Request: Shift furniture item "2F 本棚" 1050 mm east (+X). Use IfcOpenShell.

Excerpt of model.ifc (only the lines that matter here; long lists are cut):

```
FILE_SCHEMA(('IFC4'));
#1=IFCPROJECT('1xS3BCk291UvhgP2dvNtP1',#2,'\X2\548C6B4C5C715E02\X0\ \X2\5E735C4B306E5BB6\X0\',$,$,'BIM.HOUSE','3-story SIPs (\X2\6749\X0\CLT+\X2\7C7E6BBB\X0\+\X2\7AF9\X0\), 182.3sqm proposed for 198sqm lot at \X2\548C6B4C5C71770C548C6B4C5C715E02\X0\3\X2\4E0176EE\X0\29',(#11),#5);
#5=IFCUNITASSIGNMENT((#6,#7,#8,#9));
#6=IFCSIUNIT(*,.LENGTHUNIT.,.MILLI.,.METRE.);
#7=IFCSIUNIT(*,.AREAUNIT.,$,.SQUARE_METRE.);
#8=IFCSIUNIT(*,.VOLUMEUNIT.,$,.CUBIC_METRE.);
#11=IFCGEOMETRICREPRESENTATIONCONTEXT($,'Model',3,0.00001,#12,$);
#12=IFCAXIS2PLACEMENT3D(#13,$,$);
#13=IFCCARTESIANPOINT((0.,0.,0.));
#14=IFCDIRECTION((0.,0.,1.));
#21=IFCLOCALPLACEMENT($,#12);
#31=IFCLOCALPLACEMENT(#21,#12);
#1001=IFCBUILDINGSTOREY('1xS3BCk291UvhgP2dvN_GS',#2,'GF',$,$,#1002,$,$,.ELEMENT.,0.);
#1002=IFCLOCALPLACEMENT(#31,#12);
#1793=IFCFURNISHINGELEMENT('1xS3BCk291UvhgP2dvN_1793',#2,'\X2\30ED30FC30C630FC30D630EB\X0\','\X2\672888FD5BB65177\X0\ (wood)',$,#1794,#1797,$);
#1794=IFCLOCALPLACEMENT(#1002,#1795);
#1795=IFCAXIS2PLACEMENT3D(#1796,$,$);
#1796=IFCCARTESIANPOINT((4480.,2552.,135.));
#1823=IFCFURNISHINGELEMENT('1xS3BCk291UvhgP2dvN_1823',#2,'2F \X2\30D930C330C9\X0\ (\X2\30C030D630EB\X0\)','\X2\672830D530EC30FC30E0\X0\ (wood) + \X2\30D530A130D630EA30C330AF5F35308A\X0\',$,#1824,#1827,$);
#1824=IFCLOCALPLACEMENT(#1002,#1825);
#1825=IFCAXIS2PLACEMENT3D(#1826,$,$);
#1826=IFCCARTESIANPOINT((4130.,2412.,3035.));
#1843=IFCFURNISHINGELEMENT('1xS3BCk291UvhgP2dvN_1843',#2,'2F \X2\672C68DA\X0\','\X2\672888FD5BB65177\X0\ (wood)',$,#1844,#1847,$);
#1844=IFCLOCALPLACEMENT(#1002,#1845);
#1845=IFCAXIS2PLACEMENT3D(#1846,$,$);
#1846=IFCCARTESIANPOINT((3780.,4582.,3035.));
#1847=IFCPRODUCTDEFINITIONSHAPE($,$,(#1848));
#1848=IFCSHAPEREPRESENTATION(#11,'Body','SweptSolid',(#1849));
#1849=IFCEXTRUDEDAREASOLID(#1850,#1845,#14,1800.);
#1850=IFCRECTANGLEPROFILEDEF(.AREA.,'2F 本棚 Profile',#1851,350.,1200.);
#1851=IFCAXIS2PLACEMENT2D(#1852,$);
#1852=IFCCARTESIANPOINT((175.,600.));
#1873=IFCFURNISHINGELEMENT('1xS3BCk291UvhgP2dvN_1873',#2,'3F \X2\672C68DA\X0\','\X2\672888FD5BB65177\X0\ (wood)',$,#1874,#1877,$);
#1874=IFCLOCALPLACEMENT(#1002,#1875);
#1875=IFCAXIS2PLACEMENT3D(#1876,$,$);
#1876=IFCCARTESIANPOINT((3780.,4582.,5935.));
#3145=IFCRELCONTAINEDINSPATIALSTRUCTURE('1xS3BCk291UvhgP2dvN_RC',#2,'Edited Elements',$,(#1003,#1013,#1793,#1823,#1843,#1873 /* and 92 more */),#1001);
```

```python
import ifcopenshell
import ifcopenshell.api.geometry
import ifcopenshell.util.placement
import ifcopenshell.util.unit

model = ifcopenshell.open("model.ifc")
unit_scale = ifcopenshell.util.unit.calculate_unit_scale(model)

item = model.by_guid("1xS3BCk291UvhgP2dvN_1843")
matrix = ifcopenshell.util.placement.get_local_placement(item.ObjectPlacement)
matrix[0, 3] += 1.05 / unit_scale
ifcopenshell.api.geometry.edit_object_placement(model, product=item, matrix=matrix, is_si=False)

print(ifcopenshell.util.placement.get_local_placement(item.ObjectPlacement).round(3) + 0.0)

model.write("model_edited.ifc")
```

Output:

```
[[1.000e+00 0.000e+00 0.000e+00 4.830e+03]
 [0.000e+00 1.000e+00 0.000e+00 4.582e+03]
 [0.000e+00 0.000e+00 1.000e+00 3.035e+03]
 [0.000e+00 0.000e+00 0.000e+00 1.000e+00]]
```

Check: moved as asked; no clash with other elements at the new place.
